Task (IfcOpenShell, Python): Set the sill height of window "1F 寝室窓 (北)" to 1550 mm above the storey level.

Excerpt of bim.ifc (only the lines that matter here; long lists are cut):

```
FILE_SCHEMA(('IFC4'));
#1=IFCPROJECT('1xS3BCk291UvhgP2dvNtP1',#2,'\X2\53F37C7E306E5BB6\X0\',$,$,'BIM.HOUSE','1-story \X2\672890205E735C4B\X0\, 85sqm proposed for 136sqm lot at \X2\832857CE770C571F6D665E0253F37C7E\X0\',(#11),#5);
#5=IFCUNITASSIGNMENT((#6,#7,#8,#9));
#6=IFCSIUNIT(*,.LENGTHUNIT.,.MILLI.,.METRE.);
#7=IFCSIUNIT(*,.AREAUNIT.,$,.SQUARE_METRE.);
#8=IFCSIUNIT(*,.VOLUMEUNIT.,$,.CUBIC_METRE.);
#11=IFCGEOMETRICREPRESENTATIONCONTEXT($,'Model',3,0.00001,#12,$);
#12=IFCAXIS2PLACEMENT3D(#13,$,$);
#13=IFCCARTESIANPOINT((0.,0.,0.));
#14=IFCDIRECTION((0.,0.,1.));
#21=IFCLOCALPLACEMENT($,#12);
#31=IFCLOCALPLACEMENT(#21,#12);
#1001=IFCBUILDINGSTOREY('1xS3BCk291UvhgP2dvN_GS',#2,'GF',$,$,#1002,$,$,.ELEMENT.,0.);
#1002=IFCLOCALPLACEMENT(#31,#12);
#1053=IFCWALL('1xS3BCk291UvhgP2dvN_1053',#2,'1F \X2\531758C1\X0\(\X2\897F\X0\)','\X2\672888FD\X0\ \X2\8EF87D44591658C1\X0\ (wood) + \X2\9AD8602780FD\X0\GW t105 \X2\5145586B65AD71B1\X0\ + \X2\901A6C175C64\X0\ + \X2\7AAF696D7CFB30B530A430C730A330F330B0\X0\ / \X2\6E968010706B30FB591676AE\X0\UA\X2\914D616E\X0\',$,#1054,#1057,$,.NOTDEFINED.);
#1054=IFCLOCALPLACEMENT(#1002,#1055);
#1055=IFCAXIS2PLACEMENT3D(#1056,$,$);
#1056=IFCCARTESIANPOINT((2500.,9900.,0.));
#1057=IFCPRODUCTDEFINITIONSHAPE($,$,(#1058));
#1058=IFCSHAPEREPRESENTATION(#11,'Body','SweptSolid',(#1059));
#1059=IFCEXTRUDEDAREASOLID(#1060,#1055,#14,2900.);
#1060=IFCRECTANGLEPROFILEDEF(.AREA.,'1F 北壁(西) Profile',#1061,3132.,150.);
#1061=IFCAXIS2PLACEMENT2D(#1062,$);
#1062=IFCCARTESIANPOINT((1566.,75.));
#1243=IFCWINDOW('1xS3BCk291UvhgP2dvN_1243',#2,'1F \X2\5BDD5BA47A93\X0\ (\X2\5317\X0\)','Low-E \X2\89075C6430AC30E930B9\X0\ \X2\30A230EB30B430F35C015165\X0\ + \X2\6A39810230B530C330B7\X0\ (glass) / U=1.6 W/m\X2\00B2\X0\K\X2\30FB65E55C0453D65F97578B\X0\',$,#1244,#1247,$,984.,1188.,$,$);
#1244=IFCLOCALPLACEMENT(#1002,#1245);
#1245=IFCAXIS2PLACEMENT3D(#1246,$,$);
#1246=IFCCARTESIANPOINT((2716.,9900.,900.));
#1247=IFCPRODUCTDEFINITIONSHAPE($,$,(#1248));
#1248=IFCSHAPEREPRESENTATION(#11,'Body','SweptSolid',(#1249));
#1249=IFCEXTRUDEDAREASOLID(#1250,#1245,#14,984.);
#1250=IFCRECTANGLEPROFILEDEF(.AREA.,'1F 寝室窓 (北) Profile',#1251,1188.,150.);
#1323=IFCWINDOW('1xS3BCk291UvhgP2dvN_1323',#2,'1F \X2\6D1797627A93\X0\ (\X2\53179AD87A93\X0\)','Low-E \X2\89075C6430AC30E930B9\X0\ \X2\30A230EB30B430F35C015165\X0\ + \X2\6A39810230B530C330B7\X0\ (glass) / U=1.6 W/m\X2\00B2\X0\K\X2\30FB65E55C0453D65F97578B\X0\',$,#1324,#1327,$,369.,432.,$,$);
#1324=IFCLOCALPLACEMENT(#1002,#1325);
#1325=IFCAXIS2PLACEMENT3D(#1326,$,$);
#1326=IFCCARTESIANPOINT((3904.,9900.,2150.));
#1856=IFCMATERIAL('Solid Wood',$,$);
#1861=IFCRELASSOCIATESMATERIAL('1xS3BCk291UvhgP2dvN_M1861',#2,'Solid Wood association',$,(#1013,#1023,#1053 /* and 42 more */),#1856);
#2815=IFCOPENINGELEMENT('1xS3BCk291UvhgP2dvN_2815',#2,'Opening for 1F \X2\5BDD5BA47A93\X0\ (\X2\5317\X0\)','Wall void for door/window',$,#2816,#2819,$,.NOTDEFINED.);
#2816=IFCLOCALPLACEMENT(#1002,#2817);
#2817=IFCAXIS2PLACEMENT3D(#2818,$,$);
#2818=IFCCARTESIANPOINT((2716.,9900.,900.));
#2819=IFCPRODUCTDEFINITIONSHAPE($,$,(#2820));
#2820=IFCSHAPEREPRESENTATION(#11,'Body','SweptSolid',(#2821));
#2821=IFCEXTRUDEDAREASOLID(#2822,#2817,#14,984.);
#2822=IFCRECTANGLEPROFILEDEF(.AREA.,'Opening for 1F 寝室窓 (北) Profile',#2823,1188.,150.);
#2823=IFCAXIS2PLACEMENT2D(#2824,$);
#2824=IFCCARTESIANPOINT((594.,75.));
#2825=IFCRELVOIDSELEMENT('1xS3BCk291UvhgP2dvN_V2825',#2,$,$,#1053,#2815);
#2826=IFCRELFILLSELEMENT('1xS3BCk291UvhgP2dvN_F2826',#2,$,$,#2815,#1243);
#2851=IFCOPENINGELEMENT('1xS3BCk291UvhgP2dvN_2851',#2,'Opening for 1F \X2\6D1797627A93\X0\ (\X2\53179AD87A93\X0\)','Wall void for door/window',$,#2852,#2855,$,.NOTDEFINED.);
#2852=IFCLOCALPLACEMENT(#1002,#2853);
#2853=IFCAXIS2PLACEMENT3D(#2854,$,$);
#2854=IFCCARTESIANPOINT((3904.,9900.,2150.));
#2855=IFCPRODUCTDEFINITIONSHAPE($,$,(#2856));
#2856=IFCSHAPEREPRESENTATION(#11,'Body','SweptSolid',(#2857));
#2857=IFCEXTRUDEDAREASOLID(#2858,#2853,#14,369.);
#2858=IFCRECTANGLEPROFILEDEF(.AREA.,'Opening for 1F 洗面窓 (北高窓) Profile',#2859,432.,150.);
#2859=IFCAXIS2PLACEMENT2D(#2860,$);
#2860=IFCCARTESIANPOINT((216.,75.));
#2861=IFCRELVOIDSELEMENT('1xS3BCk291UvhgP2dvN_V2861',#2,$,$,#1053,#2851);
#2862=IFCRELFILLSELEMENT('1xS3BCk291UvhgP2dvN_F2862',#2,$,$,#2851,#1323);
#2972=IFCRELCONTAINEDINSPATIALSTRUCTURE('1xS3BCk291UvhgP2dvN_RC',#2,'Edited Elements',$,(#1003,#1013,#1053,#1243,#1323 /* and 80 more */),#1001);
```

```python
import numpy as np
import ifcopenshell
import ifcopenshell.api.geometry
import ifcopenshell.geom
import ifcopenshell.util.element
import ifcopenshell.util.placement
import ifcopenshell.util.shape
import ifcopenshell.util.unit

model = ifcopenshell.open("bim.ifc")
unit_scale = ifcopenshell.util.unit.calculate_unit_scale(model)

window = model.by_guid("1xS3BCk291UvhgP2dvN_1243")
opening = window.FillsVoids[0].RelatingOpeningElement
storey = ifcopenshell.util.element.get_container(window, ifc_class="IfcBuildingStorey")
level = ifcopenshell.util.placement.get_local_placement(storey.ObjectPlacement)[2, 3]

# The opening's origin need not be at the sill, so measure its lowest point.
shape = ifcopenshell.geom.create_shape(ifcopenshell.geom.settings(), opening)
bottom = ifcopenshell.util.shape.get_shape_bottom_elevation(shape, shape.geometry) / unit_scale
dz = level + 1.55 / unit_scale - bottom

shift = np.array([0.0, 0.0, dz])
# The window is not placed relative to its opening, so move both.
for product in (opening, window):
    matrix = ifcopenshell.util.placement.get_local_placement(product.ObjectPlacement)
    matrix[:3, 3] += shift
    ifcopenshell.api.geometry.edit_object_placement(model, product=product, matrix=matrix, is_si=False)

print(f"moved by {dz * unit_scale:+.3f} m")

model.write("bim_updated.ifc")
```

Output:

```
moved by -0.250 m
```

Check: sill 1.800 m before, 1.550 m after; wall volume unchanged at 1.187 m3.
